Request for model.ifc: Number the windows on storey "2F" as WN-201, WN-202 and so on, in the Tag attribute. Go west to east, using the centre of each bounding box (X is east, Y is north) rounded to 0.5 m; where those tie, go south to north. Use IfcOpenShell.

First a look at what the model holds.

```python
import ifcopenshell
import ifcopenshell.util.element
import ifcopenshell.util.placement

model = ifcopenshell.open("model.ifc")
print(model.schema)
storey = next(s for s in model.by_type("IfcBuildingStorey") if s.Name == "2F")
windows = [e for e in ifcopenshell.util.element.get_decomposition(storey) if e.is_a("IfcWindow")]
for e in sorted(windows, key=lambda e: e.id()):
    origin = ifcopenshell.util.placement.get_local_placement(e.ObjectPlacement)[:3, 3]
    print(e.id(), e.Tag, e.Name, origin.round(2) + 0.0, sep=" | ")
```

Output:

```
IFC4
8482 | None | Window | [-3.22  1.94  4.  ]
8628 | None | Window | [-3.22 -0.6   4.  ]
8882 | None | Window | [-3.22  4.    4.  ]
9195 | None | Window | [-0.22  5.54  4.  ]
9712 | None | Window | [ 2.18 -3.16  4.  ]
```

```python
import ifcopenshell
import ifcopenshell.geom
import ifcopenshell.util.element
import ifcopenshell.util.shape

model = ifcopenshell.open("model.ifc")
settings = ifcopenshell.geom.settings()
settings.set("use-world-coords", True)


def centre(element):
    shape = ifcopenshell.geom.create_shape(settings, element)
    return ifcopenshell.util.shape.get_bbox_centroid(shape.geometry)


storey = next(s for s in model.by_type("IfcBuildingStorey") if s.Name == "2F")
windows = [e for e in ifcopenshell.util.element.get_decomposition(storey) if e.is_a("IfcWindow")]

# Insertion points can sit at a corner or the storey origin, so sort by the geometry (in metres).
centres = {e: centre(e) for e in windows}
windows.sort(key=lambda e: (round(centres[e][0] / 0.5), centres[e][1]))

for i, e in enumerate(windows, start=1):
    number = f"WN-2{i:02d}"
    e.Tag = number
    print(e.id(), number)

model.write("model_rev.ifc")
```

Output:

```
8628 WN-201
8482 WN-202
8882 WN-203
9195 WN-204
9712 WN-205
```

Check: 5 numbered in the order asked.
